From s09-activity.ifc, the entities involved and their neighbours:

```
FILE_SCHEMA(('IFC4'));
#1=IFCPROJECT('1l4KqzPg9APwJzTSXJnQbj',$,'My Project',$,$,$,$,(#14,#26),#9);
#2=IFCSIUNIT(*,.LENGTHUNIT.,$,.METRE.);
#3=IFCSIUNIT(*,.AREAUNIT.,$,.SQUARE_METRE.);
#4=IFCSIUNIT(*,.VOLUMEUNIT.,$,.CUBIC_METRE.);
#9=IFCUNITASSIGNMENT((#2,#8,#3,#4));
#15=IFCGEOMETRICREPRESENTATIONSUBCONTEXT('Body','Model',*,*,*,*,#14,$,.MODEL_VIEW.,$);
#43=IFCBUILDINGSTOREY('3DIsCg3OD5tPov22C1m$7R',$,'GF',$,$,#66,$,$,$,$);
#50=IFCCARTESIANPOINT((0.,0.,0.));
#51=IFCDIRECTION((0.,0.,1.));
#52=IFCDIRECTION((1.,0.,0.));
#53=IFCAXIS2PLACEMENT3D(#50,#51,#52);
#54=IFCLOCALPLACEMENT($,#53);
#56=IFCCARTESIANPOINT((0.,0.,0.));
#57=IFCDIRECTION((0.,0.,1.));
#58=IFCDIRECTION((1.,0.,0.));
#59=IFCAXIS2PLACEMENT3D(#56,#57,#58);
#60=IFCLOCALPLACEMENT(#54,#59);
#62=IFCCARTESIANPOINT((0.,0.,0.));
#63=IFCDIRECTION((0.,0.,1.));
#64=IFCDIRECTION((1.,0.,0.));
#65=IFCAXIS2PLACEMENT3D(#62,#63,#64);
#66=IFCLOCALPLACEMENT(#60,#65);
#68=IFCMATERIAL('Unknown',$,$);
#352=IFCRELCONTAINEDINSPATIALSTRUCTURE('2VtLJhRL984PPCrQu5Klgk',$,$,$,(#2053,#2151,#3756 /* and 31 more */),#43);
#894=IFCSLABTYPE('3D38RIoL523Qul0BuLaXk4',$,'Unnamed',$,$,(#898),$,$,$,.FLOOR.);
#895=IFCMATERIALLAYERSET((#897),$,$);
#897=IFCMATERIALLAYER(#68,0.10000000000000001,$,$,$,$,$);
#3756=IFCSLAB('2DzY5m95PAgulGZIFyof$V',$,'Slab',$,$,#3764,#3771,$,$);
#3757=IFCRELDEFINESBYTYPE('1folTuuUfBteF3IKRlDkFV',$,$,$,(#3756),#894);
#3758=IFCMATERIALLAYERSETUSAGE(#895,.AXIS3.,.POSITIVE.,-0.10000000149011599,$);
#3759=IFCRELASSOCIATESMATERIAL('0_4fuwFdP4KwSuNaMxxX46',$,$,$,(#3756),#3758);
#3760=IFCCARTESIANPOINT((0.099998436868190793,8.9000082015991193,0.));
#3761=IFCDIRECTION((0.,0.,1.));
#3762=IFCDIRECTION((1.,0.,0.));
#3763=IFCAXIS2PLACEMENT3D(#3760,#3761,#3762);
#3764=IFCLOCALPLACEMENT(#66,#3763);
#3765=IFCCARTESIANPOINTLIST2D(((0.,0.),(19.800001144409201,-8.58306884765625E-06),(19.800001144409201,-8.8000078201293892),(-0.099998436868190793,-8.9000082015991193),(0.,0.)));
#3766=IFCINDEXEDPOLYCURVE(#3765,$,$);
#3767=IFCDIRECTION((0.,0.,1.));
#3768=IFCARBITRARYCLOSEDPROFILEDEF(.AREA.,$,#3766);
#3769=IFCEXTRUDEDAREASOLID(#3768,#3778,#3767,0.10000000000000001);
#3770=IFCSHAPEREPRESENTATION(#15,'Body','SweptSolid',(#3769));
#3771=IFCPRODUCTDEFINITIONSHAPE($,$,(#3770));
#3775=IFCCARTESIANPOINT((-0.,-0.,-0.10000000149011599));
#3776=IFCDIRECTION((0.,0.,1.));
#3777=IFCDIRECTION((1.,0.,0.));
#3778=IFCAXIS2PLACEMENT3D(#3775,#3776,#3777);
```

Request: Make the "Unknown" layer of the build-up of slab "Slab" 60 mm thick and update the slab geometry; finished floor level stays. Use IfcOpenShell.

```python
import ifcopenshell
import ifcopenshell.util.element
import ifcopenshell.util.representation
import ifcopenshell.util.unit

model = ifcopenshell.open("s09-activity.ifc")
unit_scale = ifcopenshell.util.unit.calculate_unit_scale(model)

layer_set = model.by_id(895)
layer = next(l for l in layer_set.MaterialLayers if l.Material and l.Material.Name == "Unknown")
change = 0.06 / unit_scale - layer.LayerThickness
layer.LayerThickness += change

# Geometry does not follow the layer set by itself.
slabs = [e for e in ifcopenshell.util.element.get_elements_by_material(model, layer_set) if e.is_a("IfcSlab")]
for slab in sorted(slabs, key=lambda e: e.id()):
    body = ifcopenshell.util.representation.get_representation(slab, "Model", "Body")
    solid = body.Items[0]
    old_depth = solid.Depth
    solid.Depth += change
    # Extruded upwards: lower the start of the extrusion so the top stays.
    x, y, z = solid.Position.Location.Coordinates
    solid.Position.Location = model.createIfcCartesianPoint((x, y, z - change))
    print(slab.id(), f"{old_depth:g} -> {solid.Depth:g}")

# The layers are counted up from the underside, which has moved.
for usage in {ifcopenshell.util.element.get_material(slab) for slab in slabs}:
    usage.OffsetFromReferenceLine -= change

model.write("s09-activity_v2.ifc")
```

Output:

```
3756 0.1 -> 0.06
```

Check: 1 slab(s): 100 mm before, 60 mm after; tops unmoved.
